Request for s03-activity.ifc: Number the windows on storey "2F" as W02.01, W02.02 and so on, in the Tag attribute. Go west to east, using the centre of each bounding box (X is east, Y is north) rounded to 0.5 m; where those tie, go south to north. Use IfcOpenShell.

First a look at what the model holds.

```python
import ifcopenshell
import ifcopenshell.util.element
import ifcopenshell.util.placement

model = ifcopenshell.open("s03-activity.ifc")
print(model.schema)
storey = next(s for s in model.by_type("IfcBuildingStorey") if s.Name == "2F")
windows = [e for e in ifcopenshell.util.element.get_decomposition(storey) if e.is_a("IfcWindow")]
for e in sorted(windows, key=lambda e: e.id()):
    origin = ifcopenshell.util.placement.get_local_placement(e.ObjectPlacement)[:3, 3]
    print(e.id(), e.Tag, e.Name, origin.round(2) + 0.0, sep=" | ")
```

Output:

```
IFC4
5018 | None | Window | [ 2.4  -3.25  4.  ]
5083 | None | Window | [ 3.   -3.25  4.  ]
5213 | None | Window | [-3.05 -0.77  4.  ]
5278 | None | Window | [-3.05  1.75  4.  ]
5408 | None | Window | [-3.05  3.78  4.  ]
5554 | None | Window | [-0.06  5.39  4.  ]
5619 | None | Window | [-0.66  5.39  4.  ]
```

```python
import ifcopenshell
import ifcopenshell.geom
import ifcopenshell.util.element
import ifcopenshell.util.shape

model = ifcopenshell.open("s03-activity.ifc")
settings = ifcopenshell.geom.settings()
settings.set("use-world-coords", True)


def centre(element):
    shape = ifcopenshell.geom.create_shape(settings, element)
    return ifcopenshell.util.shape.get_bbox_centroid(shape.geometry)


storey = next(s for s in model.by_type("IfcBuildingStorey") if s.Name == "2F")
windows = [e for e in ifcopenshell.util.element.get_decomposition(storey) if e.is_a("IfcWindow")]

# Insertion points can sit at a corner or the storey origin, so sort by the geometry (in metres).
centres = {e: centre(e) for e in windows}
windows.sort(key=lambda e: (round(centres[e][0] / 0.5), centres[e][1]))

for i, e in enumerate(windows, start=1):
    number = f"W02.{i:02d}"
    e.Tag = number
    print(e.id(), number)

model.write("s03-activity_v2.ifc")
```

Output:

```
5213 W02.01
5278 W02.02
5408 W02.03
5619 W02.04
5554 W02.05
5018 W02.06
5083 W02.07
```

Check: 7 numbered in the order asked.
